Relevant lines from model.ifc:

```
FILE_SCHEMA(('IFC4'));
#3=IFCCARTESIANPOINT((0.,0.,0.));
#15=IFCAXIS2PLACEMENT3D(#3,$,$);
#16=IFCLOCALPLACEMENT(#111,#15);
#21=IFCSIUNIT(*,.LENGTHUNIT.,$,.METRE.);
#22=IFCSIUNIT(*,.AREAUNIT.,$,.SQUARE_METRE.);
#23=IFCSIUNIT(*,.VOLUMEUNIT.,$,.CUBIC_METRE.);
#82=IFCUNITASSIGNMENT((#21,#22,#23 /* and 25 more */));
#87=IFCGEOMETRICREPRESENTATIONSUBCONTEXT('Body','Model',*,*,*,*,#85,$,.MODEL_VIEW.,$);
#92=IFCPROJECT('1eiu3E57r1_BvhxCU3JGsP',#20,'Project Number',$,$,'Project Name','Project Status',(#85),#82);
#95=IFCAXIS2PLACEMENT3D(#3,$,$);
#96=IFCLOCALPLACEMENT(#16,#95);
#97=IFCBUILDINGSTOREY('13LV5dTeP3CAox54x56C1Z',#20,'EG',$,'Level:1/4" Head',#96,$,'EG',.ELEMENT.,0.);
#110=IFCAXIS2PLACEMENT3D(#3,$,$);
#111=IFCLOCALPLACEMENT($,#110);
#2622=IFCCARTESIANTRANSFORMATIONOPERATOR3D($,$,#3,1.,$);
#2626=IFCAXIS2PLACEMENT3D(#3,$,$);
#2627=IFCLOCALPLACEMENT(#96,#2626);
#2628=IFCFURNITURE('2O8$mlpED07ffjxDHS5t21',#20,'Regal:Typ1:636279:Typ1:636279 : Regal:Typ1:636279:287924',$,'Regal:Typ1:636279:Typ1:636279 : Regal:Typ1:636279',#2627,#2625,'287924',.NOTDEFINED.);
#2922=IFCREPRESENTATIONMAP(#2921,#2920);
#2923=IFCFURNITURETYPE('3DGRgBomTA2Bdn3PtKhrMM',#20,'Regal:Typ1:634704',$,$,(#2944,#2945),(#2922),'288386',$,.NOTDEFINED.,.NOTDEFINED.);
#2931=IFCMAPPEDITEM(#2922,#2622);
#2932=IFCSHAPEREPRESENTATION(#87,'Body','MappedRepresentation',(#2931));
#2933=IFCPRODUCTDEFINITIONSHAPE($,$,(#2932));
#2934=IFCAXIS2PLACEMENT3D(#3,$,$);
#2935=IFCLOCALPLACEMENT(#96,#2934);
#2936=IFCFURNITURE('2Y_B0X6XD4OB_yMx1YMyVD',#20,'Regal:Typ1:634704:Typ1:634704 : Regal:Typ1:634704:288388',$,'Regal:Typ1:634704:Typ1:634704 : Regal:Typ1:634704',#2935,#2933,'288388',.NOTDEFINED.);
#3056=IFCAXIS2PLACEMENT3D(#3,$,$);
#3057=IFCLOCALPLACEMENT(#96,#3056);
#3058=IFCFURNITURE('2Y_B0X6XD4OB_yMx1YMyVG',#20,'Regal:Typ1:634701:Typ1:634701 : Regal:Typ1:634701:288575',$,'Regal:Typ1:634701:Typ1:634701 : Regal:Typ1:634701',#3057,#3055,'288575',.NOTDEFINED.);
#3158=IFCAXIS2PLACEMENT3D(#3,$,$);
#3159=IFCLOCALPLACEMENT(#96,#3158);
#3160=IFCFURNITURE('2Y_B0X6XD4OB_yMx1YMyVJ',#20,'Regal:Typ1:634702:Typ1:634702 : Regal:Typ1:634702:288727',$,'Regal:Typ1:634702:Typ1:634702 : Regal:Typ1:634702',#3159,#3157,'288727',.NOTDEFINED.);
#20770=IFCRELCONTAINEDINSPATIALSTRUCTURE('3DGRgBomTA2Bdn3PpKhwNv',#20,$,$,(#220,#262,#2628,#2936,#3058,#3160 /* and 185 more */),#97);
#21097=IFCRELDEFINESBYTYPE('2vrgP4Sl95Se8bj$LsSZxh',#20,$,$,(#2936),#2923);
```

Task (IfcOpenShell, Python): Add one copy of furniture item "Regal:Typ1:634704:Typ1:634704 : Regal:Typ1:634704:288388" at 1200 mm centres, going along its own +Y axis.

```python
import ifcopenshell
import ifcopenshell.api.geometry
import ifcopenshell.api.root
import ifcopenshell.util.element
import ifcopenshell.util.placement
import ifcopenshell.util.unit

model = ifcopenshell.open("model.ifc")
unit_scale = ifcopenshell.util.unit.calculate_unit_scale(model)


def reuse_history(source, copy):
    """copy_class also copies each property set's owner history, people and application; keep the originals."""
    for rel in copy.IsDefinedBy:
        if rel.is_a("IfcRelDefinesByProperties") and (history := rel.RelatingPropertyDefinition.OwnerHistory):
            rel.RelatingPropertyDefinition.OwnerHistory = source.OwnerHistory
            ifcopenshell.util.element.remove_deep2(model, history)


source = model.by_guid("2Y_B0X6XD4OB_yMx1YMyVD")
base = ifcopenshell.util.placement.get_local_placement(source.ObjectPlacement)
step = base[:3, 1] * 1.2 / unit_scale

for i in range(1, 2):
    copy = ifcopenshell.api.root.copy_class(model, product=source)
    copy.Representation = ifcopenshell.util.element.copy_deep(
        model, source.Representation, exclude=["IfcGeometricRepresentationContext", "IfcRepresentationMap"]
    )
    copy.Name = "Regal:Typ1:634704:Typ1:634704 : Regal:Typ1"
    copy.Tag = None
    reuse_history(source, copy)
    matrix = base.copy()
    matrix[:3, 3] += i * step
    print("added at", matrix[:3, 3].round(3) + 0.0)
    ifcopenshell.api.geometry.edit_object_placement(model, product=copy, matrix=matrix, is_si=False)

model.write("model_edited.ifc")
```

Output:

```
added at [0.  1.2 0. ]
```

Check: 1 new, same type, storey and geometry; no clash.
